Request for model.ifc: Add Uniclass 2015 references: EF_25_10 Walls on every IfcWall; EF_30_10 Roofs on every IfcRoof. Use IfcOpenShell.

First a look at what the model holds.

```python
import ifcopenshell

model = ifcopenshell.open("model.ifc")
print(model.schema)
print("classifications:", [c.Name for c in model.by_type("IfcClassification")])
for ifc_class in ("IfcDoor", "IfcRoof", "IfcStair", "IfcWall", "IfcWindow"):
    print(ifc_class, len(model.by_type(ifc_class)))
```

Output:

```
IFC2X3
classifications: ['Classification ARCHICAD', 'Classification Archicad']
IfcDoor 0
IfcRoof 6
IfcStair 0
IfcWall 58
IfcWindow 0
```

```python
import ifcopenshell
import ifcopenshell.api.classification

model = ifcopenshell.open("model.ifc")

# IFC2X3 requires Source and Edition and has no link from the project to the system.
system = model.create_entity("IfcClassification", Source="NBS", Edition="2015", Name="Uniclass 2015")

codes = {
    "IfcWall": ("EF_25_10", "Walls"),
    "IfcRoof": ("EF_30_10", "Roofs"),
}
for ifc_class, (code, name) in codes.items():
    products = model.by_type(ifc_class)
    ifcopenshell.api.classification.add_reference(
        model, products=products, classification=system, identification=code, name=name
    )
    print(code, len(products))

model.write("model_rev.ifc")
```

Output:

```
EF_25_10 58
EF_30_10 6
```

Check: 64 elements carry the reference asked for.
